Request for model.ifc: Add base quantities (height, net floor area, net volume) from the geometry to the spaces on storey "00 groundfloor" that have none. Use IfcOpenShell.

First a look at what the model holds.

```python
import ifcopenshell
import ifcopenshell.util.element
import ifcopenshell.util.unit

model = ifcopenshell.open("model.ifc")
print(model.schema)
for unit_type in ("LENGTHUNIT", "AREAUNIT", "VOLUMEUNIT"):
    print(unit_type, ifcopenshell.util.unit.calculate_unit_scale(model, unit_type))
storey = next(s for s in model.by_type("IfcBuildingStorey") if s.Name == "00 groundfloor")
spaces = [e for e in ifcopenshell.util.element.get_decomposition(storey) if e.is_a("IfcSpace")]
for e in sorted(spaces, key=lambda e: e.id()):
    print(e.id(), e.is_a(), e.Name, list(ifcopenshell.util.element.get_psets(e, qtos_only=True)), sep=" | ")
```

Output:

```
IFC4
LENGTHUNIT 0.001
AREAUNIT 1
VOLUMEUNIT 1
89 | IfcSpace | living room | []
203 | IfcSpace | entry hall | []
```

```python
import ifcopenshell
import ifcopenshell.api.pset
import ifcopenshell.geom
import ifcopenshell.util.element
import ifcopenshell.util.shape
import ifcopenshell.util.unit

model = ifcopenshell.open("model.ifc")
unit_scale = ifcopenshell.util.unit.calculate_unit_scale(model)
area_scale = ifcopenshell.util.unit.calculate_unit_scale(model, "AREAUNIT")
volume_scale = ifcopenshell.util.unit.calculate_unit_scale(model, "VOLUMEUNIT")
settings = ifcopenshell.geom.settings()

storey = next(s for s in model.by_type("IfcBuildingStorey") if s.Name == "00 groundfloor")
spaces = [e for e in ifcopenshell.util.element.get_decomposition(storey) if e.is_a("IfcSpace")]

for e in sorted(spaces, key=lambda e: e.id()):
    if ifcopenshell.util.element.get_psets(e, qtos_only=True, should_inherit=False):
        continue
    # Geometry comes back in metres, in the element's own axes.
    shape = ifcopenshell.geom.create_shape(settings, e)
    values = {
        "Height": ifcopenshell.util.shape.get_z(shape.geometry) / unit_scale,
        "NetFloorArea": ifcopenshell.util.shape.get_footprint_area(shape.geometry) / area_scale,
        "NetVolume": ifcopenshell.util.shape.get_volume(shape.geometry) / volume_scale,
    }
    qto = ifcopenshell.api.pset.add_qto(model, product=e, name="Qto_SpaceBaseQuantities")
    ifcopenshell.api.pset.edit_qto(model, qto=qto, properties=values)
    print(e.id(), {k: round(v, 3) for k, v in values.items()})

model.write("model_v2.ifc")
```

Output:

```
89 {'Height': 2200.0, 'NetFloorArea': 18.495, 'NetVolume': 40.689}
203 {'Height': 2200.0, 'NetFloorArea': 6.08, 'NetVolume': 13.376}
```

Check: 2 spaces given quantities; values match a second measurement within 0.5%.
